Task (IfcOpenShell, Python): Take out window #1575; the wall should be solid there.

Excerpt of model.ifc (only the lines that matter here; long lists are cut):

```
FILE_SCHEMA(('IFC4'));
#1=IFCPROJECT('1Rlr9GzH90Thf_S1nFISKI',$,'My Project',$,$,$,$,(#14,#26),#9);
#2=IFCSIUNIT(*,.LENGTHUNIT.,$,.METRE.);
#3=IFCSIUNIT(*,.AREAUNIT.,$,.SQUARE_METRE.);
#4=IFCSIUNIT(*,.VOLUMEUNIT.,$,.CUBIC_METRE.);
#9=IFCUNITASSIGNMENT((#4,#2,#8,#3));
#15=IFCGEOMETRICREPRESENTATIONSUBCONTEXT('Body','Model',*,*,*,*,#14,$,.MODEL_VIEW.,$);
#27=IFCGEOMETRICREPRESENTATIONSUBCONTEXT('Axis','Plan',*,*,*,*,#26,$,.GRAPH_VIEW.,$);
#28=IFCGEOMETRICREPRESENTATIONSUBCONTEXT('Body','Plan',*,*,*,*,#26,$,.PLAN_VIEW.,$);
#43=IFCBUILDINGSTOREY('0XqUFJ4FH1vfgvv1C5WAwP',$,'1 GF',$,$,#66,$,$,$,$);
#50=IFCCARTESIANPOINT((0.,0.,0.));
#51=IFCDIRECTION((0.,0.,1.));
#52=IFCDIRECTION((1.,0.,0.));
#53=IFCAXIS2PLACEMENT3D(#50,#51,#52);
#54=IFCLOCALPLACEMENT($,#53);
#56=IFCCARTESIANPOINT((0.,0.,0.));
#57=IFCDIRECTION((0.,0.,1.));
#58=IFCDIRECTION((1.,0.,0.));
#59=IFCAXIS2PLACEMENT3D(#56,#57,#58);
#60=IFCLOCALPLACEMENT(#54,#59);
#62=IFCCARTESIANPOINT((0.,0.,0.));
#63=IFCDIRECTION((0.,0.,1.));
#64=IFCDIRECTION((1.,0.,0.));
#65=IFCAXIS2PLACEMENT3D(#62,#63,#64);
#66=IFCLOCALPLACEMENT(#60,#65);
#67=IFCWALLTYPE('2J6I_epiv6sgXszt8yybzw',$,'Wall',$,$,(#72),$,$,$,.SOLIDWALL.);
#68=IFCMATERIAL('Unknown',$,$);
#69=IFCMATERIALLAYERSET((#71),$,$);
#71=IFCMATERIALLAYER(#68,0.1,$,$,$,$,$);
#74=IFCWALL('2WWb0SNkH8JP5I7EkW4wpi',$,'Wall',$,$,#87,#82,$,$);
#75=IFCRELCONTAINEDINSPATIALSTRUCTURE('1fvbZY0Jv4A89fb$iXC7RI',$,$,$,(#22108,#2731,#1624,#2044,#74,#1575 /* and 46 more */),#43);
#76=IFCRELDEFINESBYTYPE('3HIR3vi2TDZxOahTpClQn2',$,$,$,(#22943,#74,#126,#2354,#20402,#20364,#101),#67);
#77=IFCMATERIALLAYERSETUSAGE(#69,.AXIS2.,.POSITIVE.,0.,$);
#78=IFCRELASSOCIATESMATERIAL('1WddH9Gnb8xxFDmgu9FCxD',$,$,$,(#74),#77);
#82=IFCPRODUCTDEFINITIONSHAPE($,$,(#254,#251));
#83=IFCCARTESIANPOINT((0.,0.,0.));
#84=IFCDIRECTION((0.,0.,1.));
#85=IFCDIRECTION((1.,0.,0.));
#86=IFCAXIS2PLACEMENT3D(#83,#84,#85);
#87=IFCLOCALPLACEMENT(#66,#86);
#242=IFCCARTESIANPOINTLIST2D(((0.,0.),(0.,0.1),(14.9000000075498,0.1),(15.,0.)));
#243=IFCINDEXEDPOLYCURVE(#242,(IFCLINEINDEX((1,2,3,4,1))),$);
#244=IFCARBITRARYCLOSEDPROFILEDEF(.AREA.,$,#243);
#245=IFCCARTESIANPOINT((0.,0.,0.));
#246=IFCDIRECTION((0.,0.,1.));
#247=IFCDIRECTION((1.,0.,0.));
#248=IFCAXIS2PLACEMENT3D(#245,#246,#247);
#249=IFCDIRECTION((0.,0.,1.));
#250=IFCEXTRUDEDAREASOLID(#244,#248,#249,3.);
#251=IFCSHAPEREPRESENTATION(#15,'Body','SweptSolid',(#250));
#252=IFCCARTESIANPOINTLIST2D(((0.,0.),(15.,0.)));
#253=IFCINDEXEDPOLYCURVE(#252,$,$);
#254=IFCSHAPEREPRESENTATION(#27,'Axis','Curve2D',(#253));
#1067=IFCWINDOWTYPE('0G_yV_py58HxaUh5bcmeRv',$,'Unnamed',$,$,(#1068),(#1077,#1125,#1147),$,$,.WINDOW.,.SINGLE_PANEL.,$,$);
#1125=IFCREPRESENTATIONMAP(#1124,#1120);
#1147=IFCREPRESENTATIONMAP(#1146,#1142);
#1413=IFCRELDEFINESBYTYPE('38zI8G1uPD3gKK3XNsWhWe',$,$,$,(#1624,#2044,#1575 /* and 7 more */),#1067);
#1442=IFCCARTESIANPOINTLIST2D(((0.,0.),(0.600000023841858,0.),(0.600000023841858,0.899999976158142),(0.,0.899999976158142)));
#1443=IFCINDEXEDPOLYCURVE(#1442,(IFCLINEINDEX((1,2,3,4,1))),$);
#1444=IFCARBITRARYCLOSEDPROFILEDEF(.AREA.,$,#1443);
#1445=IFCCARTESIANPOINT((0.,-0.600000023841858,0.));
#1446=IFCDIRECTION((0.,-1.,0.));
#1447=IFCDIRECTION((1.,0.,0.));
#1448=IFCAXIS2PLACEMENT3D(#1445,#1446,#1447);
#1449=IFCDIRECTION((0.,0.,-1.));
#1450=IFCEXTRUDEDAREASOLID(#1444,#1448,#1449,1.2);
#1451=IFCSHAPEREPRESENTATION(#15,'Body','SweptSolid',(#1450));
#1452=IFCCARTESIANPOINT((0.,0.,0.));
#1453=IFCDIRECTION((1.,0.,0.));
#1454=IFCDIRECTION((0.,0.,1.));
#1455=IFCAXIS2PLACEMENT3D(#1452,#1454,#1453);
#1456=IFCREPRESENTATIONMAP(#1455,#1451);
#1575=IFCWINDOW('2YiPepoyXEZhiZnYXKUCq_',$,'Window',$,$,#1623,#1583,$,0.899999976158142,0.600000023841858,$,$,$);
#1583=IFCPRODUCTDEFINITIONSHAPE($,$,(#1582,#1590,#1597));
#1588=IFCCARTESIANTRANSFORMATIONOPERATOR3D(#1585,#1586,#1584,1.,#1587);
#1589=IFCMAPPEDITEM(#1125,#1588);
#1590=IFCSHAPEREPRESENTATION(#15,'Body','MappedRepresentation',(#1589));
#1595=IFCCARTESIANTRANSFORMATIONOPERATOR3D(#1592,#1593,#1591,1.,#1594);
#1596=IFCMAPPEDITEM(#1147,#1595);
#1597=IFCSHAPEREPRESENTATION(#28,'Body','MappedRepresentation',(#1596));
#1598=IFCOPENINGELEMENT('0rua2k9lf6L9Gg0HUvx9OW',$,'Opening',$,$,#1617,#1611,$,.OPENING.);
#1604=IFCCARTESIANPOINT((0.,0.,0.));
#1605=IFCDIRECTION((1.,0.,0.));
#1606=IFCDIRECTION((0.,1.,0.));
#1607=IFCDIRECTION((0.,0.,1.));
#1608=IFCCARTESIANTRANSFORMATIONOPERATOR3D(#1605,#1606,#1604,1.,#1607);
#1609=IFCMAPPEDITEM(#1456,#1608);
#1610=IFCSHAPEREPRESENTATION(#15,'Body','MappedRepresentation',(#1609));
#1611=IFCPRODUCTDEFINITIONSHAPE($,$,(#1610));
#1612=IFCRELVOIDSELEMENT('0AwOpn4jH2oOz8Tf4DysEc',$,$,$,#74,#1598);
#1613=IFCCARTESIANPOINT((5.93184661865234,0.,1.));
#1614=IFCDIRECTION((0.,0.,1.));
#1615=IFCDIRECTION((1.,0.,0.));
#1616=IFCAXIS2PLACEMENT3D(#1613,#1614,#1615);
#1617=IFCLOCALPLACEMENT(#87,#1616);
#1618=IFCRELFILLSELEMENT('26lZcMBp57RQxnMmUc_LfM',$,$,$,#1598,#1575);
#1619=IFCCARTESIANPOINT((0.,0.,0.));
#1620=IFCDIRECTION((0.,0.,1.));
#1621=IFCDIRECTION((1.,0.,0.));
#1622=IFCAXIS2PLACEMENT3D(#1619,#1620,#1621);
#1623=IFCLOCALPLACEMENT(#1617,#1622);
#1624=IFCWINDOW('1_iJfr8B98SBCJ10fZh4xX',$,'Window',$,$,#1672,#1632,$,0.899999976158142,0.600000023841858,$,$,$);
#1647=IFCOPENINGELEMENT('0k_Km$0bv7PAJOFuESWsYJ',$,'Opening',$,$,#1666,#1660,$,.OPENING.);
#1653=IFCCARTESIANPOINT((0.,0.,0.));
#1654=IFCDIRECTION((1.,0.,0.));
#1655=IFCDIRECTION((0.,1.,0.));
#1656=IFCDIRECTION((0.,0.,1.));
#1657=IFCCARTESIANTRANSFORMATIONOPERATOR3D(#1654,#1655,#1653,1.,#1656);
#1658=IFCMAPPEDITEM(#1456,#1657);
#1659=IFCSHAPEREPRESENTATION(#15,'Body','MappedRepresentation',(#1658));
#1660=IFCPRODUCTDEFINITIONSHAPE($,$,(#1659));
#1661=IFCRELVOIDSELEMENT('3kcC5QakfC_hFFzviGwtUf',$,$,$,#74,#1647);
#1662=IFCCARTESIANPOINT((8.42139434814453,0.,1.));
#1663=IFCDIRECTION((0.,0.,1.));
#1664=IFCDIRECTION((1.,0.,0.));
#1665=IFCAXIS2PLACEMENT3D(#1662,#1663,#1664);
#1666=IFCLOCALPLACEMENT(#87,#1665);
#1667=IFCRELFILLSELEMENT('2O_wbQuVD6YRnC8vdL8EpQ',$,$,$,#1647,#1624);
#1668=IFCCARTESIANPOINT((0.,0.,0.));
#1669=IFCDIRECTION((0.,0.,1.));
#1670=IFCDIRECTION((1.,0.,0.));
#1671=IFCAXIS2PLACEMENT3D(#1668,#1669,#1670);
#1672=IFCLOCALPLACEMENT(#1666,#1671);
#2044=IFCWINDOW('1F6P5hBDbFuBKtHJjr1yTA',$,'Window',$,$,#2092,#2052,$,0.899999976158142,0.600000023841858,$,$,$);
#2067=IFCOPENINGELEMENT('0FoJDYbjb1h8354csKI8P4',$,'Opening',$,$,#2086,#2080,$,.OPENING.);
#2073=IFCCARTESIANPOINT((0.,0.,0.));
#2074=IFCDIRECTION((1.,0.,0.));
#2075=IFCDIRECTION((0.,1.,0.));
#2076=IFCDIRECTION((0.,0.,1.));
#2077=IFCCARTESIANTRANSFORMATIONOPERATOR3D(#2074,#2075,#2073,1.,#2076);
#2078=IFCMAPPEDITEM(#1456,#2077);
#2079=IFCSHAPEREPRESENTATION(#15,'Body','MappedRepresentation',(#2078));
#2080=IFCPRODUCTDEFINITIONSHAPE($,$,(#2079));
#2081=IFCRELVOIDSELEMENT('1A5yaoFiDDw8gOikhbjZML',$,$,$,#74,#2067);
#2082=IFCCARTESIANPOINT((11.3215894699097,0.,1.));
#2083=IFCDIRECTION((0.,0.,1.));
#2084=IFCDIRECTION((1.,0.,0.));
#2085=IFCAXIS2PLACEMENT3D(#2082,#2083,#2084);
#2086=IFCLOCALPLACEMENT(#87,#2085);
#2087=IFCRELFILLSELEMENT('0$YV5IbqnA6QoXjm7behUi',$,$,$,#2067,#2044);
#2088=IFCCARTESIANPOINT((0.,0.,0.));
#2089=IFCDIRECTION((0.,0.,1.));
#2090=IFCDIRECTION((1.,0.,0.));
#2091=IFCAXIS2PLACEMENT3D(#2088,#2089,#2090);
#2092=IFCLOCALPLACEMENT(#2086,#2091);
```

```python
import ifcopenshell
import ifcopenshell.api.feature
import ifcopenshell.api.root
import ifcopenshell.geom
import ifcopenshell.util.shape

model = ifcopenshell.open("model.ifc")
settings = ifcopenshell.geom.settings()


def volume(element):
    """Net volume in cubic metres, openings subtracted."""
    shape = ifcopenshell.geom.create_shape(settings, element)
    return ifcopenshell.util.shape.get_volume(shape.geometry)


window = model.by_id(1575)
opening = window.FillsVoids[0].RelatingOpeningElement
wall = opening.VoidsElements[0].RelatingBuildingElement
before = volume(wall)

ifcopenshell.api.root.remove_product(model, product=window)
ifcopenshell.api.feature.remove_feature(model, feature=opening)

after = volume(wall)

print(f"wall volume {before:.3f} -> {after:.3f} m3")

model.write("model-out.ifc")
```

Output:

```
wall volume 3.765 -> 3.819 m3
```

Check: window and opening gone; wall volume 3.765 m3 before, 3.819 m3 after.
